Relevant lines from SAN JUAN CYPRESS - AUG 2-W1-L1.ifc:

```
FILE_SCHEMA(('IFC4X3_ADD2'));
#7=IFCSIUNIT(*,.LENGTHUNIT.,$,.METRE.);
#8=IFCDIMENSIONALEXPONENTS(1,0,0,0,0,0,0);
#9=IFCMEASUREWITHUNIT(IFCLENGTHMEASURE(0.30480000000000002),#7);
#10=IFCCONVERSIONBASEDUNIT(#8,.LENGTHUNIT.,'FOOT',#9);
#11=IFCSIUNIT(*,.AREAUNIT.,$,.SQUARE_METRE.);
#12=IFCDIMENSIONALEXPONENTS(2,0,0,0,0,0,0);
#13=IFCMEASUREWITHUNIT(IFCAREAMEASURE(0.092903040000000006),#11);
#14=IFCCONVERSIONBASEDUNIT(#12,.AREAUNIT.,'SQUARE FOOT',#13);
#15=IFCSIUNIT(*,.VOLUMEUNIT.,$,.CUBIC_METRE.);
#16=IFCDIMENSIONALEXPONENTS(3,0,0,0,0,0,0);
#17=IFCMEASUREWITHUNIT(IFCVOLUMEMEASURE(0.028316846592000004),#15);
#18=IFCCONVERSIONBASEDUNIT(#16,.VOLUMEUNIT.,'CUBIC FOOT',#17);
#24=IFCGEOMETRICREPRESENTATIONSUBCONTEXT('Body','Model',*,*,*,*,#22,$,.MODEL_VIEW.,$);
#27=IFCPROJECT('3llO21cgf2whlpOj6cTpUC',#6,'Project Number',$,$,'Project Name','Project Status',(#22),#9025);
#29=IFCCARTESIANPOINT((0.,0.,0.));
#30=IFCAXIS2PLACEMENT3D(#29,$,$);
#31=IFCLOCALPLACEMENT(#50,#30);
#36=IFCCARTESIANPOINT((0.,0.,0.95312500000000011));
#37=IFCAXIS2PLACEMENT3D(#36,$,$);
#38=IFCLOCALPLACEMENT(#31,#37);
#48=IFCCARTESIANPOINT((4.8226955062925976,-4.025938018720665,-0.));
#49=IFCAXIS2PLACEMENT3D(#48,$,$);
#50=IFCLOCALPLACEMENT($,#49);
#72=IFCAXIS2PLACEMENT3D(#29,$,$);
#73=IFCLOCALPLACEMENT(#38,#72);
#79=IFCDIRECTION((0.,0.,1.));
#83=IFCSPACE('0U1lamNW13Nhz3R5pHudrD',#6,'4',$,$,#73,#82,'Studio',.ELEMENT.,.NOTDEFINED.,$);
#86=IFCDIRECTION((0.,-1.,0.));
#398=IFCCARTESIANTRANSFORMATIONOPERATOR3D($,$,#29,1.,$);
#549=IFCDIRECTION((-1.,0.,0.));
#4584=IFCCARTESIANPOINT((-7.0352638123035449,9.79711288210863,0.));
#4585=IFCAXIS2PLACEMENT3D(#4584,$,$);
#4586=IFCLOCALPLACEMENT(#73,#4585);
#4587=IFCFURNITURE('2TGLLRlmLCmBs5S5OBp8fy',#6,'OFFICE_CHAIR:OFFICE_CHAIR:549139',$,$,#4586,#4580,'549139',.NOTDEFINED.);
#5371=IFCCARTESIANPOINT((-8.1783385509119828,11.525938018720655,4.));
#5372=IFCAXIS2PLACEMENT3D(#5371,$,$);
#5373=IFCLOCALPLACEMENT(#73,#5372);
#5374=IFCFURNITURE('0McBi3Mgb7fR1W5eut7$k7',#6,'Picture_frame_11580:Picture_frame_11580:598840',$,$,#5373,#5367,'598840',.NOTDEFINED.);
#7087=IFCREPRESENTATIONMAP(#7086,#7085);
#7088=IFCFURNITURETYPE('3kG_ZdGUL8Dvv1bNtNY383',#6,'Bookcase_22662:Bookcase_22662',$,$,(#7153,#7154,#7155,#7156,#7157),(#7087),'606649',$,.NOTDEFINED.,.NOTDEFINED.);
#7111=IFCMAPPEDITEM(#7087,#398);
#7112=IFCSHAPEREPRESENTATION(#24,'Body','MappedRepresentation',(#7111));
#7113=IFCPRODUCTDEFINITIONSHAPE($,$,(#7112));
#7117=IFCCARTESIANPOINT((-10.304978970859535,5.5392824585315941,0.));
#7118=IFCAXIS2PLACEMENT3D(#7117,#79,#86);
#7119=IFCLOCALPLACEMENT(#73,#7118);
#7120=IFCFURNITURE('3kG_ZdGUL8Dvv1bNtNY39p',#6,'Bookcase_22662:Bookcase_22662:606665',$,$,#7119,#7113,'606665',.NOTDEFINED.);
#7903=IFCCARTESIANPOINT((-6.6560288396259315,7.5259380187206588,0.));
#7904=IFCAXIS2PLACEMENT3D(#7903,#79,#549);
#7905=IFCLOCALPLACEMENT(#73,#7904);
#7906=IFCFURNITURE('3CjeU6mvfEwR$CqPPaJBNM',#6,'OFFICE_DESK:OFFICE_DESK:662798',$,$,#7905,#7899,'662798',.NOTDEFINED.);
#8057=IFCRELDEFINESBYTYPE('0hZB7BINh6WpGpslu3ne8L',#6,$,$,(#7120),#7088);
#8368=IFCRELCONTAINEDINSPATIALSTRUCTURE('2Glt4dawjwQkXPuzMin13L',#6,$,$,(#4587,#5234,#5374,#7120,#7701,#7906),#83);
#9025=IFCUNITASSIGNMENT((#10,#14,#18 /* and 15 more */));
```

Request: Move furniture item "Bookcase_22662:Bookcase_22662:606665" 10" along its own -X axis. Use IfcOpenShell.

```python
import ifcopenshell
import ifcopenshell.api.geometry
import ifcopenshell.util.placement
import ifcopenshell.util.unit

model = ifcopenshell.open("SAN JUAN CYPRESS - AUG 2-W1-L1.ifc")
unit_scale = ifcopenshell.util.unit.calculate_unit_scale(model)

item = model.by_guid("3kG_ZdGUL8Dvv1bNtNY39p")
matrix = ifcopenshell.util.placement.get_local_placement(item.ObjectPlacement)
matrix[:3, 3] -= matrix[:3, 0] * 10 * 0.0254 / unit_scale
ifcopenshell.api.geometry.edit_object_placement(model, product=item, matrix=matrix, is_si=False)

print(ifcopenshell.util.placement.get_local_placement(item.ObjectPlacement).round(3) + 0.0)

model.write("SAN JUAN CYPRESS - AUG 2-W1-L1_updated.ifc")
```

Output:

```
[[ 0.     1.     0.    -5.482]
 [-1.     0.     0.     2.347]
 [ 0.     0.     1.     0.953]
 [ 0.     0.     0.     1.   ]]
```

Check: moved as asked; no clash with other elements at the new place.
